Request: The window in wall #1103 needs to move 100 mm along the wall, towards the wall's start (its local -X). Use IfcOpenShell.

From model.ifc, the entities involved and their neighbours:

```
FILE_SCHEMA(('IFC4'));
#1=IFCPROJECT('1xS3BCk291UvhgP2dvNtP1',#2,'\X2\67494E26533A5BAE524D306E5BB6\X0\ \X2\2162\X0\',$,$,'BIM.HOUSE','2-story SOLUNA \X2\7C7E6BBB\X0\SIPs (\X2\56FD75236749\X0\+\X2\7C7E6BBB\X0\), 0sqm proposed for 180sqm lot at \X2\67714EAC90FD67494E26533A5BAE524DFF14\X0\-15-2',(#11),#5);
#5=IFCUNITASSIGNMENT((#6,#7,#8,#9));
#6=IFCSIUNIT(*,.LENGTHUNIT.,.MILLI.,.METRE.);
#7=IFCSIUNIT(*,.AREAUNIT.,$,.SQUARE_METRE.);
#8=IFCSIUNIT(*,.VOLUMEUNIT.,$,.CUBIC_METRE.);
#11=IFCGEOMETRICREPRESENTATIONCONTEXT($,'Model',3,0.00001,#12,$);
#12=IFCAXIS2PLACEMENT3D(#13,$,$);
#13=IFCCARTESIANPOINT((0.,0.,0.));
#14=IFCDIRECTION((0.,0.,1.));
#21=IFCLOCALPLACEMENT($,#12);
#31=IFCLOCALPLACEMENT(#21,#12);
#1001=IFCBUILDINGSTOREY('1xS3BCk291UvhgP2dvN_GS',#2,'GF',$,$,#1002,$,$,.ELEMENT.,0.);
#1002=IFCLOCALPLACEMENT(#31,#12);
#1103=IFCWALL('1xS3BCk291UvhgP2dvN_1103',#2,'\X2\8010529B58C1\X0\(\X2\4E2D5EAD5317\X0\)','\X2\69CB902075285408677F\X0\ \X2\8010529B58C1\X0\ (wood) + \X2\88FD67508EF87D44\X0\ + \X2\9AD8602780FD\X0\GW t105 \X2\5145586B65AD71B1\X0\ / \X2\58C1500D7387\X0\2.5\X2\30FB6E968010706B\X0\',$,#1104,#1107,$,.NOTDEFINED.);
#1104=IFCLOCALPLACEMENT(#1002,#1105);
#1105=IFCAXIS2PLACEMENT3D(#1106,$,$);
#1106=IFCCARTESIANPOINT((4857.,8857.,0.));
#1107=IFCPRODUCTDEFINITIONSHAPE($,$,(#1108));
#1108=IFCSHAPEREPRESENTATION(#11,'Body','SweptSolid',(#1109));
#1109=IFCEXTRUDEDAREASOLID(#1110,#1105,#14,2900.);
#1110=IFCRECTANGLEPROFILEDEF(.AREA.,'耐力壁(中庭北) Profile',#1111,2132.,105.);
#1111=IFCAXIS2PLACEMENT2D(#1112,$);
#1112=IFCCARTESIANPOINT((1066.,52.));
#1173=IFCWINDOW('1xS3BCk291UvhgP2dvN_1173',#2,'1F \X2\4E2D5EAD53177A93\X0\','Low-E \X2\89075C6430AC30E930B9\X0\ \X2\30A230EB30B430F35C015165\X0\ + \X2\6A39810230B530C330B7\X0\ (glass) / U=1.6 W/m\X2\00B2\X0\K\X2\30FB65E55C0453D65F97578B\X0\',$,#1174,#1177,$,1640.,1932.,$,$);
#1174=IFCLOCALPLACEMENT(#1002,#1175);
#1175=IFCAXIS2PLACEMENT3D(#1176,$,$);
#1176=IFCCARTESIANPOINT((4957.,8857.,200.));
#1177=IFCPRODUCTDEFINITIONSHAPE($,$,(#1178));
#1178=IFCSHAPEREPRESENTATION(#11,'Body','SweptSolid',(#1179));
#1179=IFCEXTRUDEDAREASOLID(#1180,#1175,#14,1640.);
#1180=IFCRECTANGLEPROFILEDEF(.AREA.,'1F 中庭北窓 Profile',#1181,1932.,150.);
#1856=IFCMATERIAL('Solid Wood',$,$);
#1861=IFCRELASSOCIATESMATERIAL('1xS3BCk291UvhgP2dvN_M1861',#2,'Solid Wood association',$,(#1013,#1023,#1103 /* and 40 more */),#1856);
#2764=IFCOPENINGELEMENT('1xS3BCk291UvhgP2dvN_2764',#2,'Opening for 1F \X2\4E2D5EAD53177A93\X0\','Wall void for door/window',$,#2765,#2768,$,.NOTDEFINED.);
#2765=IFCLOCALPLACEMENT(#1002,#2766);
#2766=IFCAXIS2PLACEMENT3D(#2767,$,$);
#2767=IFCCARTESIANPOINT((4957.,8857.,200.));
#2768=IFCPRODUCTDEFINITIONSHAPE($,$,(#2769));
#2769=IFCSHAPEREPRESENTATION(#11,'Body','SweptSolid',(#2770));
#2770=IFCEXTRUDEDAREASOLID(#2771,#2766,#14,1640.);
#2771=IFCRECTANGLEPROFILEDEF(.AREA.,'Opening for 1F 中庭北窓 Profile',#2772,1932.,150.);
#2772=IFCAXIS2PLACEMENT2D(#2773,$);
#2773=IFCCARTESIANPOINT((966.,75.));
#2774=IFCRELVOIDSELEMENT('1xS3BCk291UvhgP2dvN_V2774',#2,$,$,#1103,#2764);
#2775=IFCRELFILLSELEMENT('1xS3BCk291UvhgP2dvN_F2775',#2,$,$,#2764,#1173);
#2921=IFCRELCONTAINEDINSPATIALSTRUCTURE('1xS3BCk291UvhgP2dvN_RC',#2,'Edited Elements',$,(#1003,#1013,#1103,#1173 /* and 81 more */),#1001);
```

```python
import ifcopenshell
import ifcopenshell.api.geometry
import ifcopenshell.util.placement
import ifcopenshell.util.unit

model = ifcopenshell.open("model.ifc")
unit_scale = ifcopenshell.util.unit.calculate_unit_scale(model)

window = model.by_id(1173)
opening = window.FillsVoids[0].RelatingOpeningElement
wall = opening.VoidsElements[0].RelatingBuildingElement

wall_matrix = ifcopenshell.util.placement.get_local_placement(wall.ObjectPlacement)
shift = wall_matrix[:3, 0] * -0.1 / unit_scale
before = ifcopenshell.util.placement.get_local_placement(window.ObjectPlacement)[:3, 3].copy()

# The window is not placed relative to its opening, so move both.
for product in (opening, window):
    matrix = ifcopenshell.util.placement.get_local_placement(product.ObjectPlacement)
    matrix[:3, 3] += shift
    ifcopenshell.api.geometry.edit_object_placement(model, product=product, matrix=matrix, is_si=False)

after = ifcopenshell.util.placement.get_local_placement(window.ObjectPlacement)[:3, 3]
print("window moved by", (after - before).round(3) + 0.0)

model.write("model_v2.ifc")
```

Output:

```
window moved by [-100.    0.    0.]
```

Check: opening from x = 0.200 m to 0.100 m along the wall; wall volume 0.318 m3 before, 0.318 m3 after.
